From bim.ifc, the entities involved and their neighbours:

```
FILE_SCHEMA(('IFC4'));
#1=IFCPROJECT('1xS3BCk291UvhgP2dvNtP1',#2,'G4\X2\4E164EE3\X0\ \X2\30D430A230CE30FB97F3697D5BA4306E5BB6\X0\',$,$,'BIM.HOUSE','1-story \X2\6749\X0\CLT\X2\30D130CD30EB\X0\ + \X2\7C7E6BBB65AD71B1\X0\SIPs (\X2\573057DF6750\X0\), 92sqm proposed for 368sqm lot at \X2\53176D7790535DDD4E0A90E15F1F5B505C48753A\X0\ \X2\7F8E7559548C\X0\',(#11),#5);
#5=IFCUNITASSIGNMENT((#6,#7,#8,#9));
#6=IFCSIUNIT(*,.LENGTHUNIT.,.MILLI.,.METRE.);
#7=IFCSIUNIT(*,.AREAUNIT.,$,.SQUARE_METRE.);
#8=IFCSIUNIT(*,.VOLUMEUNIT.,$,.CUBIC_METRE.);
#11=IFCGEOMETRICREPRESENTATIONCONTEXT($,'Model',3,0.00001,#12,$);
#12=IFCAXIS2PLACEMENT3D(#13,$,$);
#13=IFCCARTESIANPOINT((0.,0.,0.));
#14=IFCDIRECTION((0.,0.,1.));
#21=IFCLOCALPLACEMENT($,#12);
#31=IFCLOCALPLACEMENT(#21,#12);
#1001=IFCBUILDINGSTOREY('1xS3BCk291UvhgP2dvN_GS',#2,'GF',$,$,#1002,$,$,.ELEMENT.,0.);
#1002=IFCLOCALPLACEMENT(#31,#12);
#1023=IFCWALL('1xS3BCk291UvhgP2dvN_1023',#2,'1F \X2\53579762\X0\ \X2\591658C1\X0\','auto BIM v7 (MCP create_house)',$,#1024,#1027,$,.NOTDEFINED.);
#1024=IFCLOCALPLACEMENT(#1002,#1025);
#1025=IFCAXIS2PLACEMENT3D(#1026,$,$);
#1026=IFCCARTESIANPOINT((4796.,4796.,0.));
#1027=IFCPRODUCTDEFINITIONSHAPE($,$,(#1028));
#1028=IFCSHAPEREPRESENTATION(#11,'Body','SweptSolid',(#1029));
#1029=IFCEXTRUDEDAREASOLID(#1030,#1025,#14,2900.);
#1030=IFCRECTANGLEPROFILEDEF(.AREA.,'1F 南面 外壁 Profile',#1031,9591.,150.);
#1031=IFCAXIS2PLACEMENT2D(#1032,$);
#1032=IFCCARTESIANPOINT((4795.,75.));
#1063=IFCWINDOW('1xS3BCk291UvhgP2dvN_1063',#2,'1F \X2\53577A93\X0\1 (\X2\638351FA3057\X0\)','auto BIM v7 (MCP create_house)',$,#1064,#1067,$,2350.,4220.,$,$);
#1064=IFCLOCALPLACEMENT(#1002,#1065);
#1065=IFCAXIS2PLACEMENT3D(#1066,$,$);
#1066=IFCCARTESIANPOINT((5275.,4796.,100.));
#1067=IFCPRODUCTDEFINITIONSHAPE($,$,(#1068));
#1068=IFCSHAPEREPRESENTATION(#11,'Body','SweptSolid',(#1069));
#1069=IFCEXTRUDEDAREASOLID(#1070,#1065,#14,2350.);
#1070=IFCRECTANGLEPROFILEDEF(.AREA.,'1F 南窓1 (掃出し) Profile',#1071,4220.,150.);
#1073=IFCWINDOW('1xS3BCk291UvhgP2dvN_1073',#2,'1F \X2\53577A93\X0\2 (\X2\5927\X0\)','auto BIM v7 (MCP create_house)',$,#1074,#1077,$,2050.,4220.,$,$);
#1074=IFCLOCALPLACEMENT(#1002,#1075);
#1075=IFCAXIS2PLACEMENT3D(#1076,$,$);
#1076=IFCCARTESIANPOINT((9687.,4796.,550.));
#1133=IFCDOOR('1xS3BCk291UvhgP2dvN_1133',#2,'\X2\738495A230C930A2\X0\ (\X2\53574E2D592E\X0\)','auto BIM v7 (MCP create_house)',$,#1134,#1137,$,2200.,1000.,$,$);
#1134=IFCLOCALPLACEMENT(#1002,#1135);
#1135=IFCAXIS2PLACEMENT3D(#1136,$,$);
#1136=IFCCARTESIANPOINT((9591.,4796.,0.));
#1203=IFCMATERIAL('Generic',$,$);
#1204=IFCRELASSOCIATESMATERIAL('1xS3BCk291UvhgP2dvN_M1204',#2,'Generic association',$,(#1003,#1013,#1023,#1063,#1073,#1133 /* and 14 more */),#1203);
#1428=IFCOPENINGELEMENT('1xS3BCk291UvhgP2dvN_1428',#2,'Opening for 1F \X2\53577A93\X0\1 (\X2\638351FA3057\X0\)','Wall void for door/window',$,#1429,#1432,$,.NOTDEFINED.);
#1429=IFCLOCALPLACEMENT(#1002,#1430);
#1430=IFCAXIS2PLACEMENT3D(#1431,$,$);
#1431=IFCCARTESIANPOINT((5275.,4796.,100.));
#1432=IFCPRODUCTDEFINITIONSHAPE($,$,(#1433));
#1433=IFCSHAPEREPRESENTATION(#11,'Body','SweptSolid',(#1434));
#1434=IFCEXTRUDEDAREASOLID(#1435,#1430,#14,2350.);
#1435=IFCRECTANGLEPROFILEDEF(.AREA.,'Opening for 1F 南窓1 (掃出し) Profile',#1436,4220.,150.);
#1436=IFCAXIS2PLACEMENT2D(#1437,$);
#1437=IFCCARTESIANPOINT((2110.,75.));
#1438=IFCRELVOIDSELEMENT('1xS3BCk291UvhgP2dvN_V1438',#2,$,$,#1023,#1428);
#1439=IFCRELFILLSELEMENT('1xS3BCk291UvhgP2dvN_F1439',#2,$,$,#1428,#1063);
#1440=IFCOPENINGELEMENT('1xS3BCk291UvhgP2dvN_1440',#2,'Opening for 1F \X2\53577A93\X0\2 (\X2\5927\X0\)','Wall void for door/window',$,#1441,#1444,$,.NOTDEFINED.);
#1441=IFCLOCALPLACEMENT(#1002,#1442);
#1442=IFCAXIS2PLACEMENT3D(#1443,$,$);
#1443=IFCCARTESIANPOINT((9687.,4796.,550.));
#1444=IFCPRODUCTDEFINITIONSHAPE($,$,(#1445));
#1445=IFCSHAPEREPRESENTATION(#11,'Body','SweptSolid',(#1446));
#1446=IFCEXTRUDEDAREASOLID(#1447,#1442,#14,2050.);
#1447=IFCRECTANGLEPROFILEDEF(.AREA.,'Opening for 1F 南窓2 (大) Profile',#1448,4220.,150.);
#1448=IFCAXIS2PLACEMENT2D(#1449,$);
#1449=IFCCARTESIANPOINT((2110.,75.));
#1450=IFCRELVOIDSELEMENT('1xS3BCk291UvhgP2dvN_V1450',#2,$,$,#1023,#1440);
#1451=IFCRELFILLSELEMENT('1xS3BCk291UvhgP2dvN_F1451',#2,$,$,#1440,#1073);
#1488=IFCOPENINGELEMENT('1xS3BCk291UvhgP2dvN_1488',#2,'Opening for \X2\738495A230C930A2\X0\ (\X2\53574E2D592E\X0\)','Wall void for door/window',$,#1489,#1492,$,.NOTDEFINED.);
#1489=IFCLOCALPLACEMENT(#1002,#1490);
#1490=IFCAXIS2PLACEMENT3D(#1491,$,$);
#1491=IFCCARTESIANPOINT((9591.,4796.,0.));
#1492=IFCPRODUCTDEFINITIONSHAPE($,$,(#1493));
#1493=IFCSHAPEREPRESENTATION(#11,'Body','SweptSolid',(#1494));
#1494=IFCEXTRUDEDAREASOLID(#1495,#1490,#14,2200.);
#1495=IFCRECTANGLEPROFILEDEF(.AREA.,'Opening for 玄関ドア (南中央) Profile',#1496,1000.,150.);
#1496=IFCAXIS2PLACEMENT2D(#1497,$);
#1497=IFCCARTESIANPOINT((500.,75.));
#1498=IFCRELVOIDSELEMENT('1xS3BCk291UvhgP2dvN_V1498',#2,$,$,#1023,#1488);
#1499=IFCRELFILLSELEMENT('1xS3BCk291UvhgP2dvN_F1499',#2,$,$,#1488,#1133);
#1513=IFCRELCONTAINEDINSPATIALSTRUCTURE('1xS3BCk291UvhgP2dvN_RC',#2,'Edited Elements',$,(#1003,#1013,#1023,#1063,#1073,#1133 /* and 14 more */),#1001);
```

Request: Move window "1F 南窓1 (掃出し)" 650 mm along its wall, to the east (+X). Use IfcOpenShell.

```python
import ifcopenshell
import ifcopenshell.api.geometry
import ifcopenshell.util.placement
import ifcopenshell.util.unit

model = ifcopenshell.open("bim.ifc")
unit_scale = ifcopenshell.util.unit.calculate_unit_scale(model)

window = model.by_guid("1xS3BCk291UvhgP2dvN_1063")
opening = window.FillsVoids[0].RelatingOpeningElement
wall = opening.VoidsElements[0].RelatingBuildingElement

wall_matrix = ifcopenshell.util.placement.get_local_placement(wall.ObjectPlacement)
shift = wall_matrix[:3, 0] * 0.65 / unit_scale
before = ifcopenshell.util.placement.get_local_placement(window.ObjectPlacement)[:3, 3].copy()

# The window is not placed relative to its opening, so move both.
for product in (opening, window):
    matrix = ifcopenshell.util.placement.get_local_placement(product.ObjectPlacement)
    matrix[:3, 3] += shift
    ifcopenshell.api.geometry.edit_object_placement(model, product=product, matrix=matrix, is_si=False)

after = ifcopenshell.util.placement.get_local_placement(window.ObjectPlacement)[:3, 3]
print("window moved by", (after - before).round(3) + 0.0)

model.write("bim-out.ifc")
```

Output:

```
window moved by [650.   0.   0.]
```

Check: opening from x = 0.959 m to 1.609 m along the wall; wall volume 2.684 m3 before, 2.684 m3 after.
